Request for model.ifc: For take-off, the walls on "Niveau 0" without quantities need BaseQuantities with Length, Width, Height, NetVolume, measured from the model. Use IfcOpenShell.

First a look at what the model holds.

```python
import ifcopenshell
import ifcopenshell.util.element
import ifcopenshell.util.unit

model = ifcopenshell.open("model.ifc")
print(model.schema)
for unit_type in ("LENGTHUNIT", "AREAUNIT", "VOLUMEUNIT"):
    print(unit_type, ifcopenshell.util.unit.calculate_unit_scale(model, unit_type))
storey = next(s for s in model.by_type("IfcBuildingStorey") if s.Name == "Niveau 0")
walls = [e for e in ifcopenshell.util.element.get_decomposition(storey) if e.is_a("IfcWall")]
for e in sorted(walls, key=lambda e: e.id()):
    print(e.id(), e.is_a(), e.Name, list(ifcopenshell.util.element.get_psets(e, qtos_only=True)), sep=" | ")
```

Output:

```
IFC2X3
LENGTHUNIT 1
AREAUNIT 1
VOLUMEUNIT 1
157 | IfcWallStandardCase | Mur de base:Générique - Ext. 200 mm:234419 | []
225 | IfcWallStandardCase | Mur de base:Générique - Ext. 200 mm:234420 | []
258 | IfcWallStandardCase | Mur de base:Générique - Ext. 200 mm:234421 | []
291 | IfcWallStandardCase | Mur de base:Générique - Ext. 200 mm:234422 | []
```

```python
import ifcopenshell
import ifcopenshell.api.pset
import ifcopenshell.geom
import ifcopenshell.util.element
import ifcopenshell.util.shape
import ifcopenshell.util.unit

model = ifcopenshell.open("model.ifc")
unit_scale = ifcopenshell.util.unit.calculate_unit_scale(model)
volume_scale = ifcopenshell.util.unit.calculate_unit_scale(model, "VOLUMEUNIT")
settings = ifcopenshell.geom.settings()

storey = next(s for s in model.by_type("IfcBuildingStorey") if s.Name == "Niveau 0")
walls = [e for e in ifcopenshell.util.element.get_decomposition(storey) if e.is_a("IfcWall")]

for e in sorted(walls, key=lambda e: e.id()):
    if ifcopenshell.util.element.get_psets(e, qtos_only=True, should_inherit=False):
        continue
    # Geometry comes back in metres, in the element's own axes.
    shape = ifcopenshell.geom.create_shape(settings, e)
    values = {
        "Length": ifcopenshell.util.shape.get_x(shape.geometry) / unit_scale,
        "Width": ifcopenshell.util.shape.get_y(shape.geometry) / unit_scale,
        "Height": ifcopenshell.util.shape.get_z(shape.geometry) / unit_scale,
        "NetVolume": ifcopenshell.util.shape.get_volume(shape.geometry) / volume_scale,
    }
    qto = ifcopenshell.api.pset.add_qto(model, product=e, name="BaseQuantities")
    ifcopenshell.api.pset.edit_qto(model, qto=qto, properties=values)
    print(e.id(), {k: round(v, 3) for k, v in values.items()})

model.write("model_updated.ifc")
```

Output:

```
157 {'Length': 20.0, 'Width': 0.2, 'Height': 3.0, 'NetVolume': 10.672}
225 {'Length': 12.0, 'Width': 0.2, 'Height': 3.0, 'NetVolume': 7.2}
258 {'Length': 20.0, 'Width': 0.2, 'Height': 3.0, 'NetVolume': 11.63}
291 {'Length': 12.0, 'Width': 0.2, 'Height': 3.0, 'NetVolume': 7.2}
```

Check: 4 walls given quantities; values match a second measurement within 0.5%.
